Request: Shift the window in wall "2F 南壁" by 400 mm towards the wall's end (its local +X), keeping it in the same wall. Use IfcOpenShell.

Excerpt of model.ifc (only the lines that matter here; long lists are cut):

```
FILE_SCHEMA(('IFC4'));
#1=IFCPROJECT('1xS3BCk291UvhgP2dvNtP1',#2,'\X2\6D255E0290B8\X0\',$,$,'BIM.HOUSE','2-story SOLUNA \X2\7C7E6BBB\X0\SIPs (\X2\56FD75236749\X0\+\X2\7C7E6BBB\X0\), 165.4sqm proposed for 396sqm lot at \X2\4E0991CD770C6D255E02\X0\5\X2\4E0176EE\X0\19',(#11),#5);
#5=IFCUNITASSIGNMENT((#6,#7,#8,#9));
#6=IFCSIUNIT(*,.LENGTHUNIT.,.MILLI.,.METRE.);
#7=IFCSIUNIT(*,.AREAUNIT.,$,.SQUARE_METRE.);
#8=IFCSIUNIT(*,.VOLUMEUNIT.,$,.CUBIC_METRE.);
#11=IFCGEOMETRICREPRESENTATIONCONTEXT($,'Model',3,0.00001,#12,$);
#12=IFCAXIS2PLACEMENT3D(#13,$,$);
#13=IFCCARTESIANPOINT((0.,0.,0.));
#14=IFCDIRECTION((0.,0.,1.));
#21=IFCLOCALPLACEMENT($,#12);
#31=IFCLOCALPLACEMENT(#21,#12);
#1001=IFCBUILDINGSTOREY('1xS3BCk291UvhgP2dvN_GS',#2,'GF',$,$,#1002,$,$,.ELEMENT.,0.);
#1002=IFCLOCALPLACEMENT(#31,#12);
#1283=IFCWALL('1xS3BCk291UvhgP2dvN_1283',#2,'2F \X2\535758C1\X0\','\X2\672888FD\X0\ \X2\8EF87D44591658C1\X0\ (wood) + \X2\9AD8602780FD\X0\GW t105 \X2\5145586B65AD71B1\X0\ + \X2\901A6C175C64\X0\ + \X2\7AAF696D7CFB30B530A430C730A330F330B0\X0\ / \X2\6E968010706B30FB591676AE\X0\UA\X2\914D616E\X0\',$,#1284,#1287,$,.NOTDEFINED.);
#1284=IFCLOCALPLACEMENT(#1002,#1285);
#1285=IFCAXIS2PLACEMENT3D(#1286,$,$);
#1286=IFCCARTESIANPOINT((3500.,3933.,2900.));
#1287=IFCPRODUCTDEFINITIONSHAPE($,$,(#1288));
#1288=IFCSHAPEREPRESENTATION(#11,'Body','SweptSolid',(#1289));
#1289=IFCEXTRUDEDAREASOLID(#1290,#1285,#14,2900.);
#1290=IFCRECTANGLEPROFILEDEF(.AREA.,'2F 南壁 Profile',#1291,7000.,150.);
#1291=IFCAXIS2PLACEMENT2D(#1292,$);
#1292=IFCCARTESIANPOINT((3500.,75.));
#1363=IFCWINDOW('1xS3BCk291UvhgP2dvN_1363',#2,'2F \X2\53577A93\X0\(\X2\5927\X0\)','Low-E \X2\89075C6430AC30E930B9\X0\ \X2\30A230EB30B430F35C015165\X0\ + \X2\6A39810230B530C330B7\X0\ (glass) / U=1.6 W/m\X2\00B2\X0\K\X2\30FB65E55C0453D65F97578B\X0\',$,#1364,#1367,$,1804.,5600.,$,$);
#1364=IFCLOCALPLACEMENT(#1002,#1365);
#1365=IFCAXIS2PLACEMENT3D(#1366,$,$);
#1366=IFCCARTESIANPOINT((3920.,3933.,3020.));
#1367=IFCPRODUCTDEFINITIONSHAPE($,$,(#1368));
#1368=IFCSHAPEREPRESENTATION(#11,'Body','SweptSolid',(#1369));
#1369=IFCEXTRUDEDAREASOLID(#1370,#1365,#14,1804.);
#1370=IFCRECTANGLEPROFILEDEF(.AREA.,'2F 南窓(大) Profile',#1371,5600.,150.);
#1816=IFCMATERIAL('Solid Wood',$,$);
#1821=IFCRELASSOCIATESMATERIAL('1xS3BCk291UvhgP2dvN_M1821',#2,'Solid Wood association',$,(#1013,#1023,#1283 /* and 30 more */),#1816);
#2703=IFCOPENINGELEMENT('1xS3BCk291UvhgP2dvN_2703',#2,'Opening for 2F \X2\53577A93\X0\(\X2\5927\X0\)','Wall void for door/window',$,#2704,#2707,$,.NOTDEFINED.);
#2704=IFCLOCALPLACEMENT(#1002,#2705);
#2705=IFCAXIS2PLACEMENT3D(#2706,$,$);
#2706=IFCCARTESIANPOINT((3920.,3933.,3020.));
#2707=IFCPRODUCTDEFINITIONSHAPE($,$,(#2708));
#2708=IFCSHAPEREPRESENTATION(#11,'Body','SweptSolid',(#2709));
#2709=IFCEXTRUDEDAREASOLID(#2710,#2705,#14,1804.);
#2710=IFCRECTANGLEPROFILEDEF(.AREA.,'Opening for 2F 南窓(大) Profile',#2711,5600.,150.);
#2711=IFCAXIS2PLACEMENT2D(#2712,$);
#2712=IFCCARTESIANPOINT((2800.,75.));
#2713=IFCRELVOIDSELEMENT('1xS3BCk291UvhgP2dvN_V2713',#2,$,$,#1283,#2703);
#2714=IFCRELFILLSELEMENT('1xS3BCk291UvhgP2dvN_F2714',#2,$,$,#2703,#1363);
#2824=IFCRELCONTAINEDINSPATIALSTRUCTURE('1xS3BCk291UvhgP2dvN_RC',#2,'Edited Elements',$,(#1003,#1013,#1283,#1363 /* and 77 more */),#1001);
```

```python
import ifcopenshell
import ifcopenshell.api.geometry
import ifcopenshell.util.placement
import ifcopenshell.util.unit

model = ifcopenshell.open("model.ifc")
unit_scale = ifcopenshell.util.unit.calculate_unit_scale(model)

window = model.by_guid("1xS3BCk291UvhgP2dvN_1363")
opening = window.FillsVoids[0].RelatingOpeningElement
wall = opening.VoidsElements[0].RelatingBuildingElement

wall_matrix = ifcopenshell.util.placement.get_local_placement(wall.ObjectPlacement)
shift = wall_matrix[:3, 0] * 0.4 / unit_scale
before = ifcopenshell.util.placement.get_local_placement(window.ObjectPlacement)[:3, 3].copy()

# The window is not placed relative to its opening, so move both.
for product in (opening, window):
    matrix = ifcopenshell.util.placement.get_local_placement(product.ObjectPlacement)
    matrix[:3, 3] += shift
    ifcopenshell.api.geometry.edit_object_placement(model, product=product, matrix=matrix, is_si=False)

after = ifcopenshell.util.placement.get_local_placement(window.ObjectPlacement)[:3, 3]
print("window moved by", (after - before).round(3) + 0.0)

model.write("model_v2.ifc")
```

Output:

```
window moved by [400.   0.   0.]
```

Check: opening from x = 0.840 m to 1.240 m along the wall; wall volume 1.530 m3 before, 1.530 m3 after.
